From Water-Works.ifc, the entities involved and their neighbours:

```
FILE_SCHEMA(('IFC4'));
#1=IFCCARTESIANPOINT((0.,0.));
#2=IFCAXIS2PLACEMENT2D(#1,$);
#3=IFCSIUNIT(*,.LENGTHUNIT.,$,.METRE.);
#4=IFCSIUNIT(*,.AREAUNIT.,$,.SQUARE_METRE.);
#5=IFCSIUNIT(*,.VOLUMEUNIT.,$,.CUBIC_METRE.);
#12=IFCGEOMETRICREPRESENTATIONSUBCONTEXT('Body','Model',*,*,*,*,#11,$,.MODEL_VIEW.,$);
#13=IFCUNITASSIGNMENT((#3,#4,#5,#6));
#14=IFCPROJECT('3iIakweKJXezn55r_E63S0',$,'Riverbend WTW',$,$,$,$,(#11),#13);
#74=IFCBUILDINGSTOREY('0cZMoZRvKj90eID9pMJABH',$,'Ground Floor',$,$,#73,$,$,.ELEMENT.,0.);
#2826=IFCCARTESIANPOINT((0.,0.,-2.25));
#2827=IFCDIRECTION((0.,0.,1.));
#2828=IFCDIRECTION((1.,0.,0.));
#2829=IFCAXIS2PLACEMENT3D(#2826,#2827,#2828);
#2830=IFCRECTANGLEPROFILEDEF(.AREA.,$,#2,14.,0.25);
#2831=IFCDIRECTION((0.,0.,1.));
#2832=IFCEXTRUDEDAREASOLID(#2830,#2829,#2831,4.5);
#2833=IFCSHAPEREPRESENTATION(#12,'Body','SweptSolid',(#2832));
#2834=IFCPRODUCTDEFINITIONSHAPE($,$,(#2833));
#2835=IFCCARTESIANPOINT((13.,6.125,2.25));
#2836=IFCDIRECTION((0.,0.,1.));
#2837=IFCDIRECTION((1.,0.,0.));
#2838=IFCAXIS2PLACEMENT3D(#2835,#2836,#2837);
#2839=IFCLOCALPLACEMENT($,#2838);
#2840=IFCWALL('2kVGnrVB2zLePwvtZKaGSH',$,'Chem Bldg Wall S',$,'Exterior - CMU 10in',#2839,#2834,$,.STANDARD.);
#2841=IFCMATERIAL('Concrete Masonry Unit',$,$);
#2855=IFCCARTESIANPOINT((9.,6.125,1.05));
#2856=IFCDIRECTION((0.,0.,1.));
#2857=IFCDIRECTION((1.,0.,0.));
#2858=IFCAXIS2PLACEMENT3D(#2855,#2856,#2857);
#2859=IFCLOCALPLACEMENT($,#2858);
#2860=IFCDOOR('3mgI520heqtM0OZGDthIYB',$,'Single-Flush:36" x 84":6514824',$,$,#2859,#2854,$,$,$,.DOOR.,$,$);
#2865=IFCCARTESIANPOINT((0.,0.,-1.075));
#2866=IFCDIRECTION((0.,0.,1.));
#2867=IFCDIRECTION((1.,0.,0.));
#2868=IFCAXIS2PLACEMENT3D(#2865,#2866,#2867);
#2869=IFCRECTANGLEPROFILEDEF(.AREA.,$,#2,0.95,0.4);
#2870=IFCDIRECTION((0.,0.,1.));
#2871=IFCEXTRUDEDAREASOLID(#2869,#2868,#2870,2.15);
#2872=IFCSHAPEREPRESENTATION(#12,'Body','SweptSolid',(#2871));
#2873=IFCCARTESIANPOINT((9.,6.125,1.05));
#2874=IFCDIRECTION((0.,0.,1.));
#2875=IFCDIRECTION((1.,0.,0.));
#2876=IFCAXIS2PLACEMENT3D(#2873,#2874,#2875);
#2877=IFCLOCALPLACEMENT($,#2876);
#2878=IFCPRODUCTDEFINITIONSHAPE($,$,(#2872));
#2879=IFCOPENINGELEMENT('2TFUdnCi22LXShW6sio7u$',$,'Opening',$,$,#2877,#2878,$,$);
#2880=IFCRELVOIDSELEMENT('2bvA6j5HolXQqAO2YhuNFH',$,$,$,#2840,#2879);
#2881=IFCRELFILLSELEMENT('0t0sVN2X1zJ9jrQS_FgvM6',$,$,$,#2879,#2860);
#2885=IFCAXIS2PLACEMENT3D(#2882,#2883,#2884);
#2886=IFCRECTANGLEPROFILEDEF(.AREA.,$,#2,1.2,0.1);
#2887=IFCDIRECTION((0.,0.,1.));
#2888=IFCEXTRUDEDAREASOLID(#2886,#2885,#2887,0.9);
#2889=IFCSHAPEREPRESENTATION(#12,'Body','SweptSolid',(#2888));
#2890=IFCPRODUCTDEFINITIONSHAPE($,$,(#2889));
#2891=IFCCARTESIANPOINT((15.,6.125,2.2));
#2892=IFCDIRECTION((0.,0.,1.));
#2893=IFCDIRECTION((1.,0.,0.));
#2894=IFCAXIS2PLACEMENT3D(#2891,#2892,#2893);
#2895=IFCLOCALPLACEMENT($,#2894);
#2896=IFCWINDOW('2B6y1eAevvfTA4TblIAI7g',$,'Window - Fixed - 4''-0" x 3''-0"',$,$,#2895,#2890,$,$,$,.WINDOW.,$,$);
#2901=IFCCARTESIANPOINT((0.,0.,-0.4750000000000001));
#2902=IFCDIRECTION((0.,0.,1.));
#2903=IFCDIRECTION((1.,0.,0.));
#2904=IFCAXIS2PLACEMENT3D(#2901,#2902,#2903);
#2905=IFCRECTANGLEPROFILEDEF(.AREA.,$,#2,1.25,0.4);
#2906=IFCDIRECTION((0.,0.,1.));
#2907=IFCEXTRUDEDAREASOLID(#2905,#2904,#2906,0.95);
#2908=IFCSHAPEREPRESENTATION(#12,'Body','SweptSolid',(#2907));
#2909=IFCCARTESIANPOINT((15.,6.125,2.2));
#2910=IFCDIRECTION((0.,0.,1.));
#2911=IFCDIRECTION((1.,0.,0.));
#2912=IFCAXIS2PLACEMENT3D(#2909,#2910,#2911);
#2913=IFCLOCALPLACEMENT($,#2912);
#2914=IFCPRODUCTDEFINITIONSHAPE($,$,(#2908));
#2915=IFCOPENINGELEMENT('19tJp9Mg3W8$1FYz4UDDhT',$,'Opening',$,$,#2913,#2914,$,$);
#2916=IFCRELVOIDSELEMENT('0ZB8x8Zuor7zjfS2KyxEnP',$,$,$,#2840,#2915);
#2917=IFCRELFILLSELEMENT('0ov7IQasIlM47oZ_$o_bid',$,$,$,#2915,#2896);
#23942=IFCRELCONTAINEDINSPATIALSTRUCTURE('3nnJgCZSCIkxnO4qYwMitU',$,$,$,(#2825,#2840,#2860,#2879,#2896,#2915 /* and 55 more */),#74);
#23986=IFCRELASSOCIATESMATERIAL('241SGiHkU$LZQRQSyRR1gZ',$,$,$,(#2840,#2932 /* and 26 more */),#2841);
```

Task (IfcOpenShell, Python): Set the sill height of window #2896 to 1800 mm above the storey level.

```python
import numpy as np
import ifcopenshell
import ifcopenshell.api.geometry
import ifcopenshell.geom
import ifcopenshell.util.element
import ifcopenshell.util.placement
import ifcopenshell.util.shape
import ifcopenshell.util.unit

model = ifcopenshell.open("Water-Works.ifc")
unit_scale = ifcopenshell.util.unit.calculate_unit_scale(model)

window = model.by_guid("2B6y1eAevvfTA4TblIAI7g")
opening = window.FillsVoids[0].RelatingOpeningElement
storey = ifcopenshell.util.element.get_container(window, ifc_class="IfcBuildingStorey")
level = ifcopenshell.util.placement.get_local_placement(storey.ObjectPlacement)[2, 3]

# The opening's origin need not be at the sill, so measure its lowest point.
shape = ifcopenshell.geom.create_shape(ifcopenshell.geom.settings(), opening)
bottom = ifcopenshell.util.shape.get_shape_bottom_elevation(shape, shape.geometry) / unit_scale
dz = level + 1.8 - bottom

shift = np.array([0.0, 0.0, dz])
# The window is not placed relative to its opening, so move both.
for product in (opening, window):
    matrix = ifcopenshell.util.placement.get_local_placement(product.ObjectPlacement)
    matrix[:3, 3] += shift
    ifcopenshell.api.geometry.edit_object_placement(model, product=product, matrix=matrix, is_si=False)

print(f"moved by {dz * unit_scale:+.3f} m")

model.write("Water-Works_edited.ifc")
```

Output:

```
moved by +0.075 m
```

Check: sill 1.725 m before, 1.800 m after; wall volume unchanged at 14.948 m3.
